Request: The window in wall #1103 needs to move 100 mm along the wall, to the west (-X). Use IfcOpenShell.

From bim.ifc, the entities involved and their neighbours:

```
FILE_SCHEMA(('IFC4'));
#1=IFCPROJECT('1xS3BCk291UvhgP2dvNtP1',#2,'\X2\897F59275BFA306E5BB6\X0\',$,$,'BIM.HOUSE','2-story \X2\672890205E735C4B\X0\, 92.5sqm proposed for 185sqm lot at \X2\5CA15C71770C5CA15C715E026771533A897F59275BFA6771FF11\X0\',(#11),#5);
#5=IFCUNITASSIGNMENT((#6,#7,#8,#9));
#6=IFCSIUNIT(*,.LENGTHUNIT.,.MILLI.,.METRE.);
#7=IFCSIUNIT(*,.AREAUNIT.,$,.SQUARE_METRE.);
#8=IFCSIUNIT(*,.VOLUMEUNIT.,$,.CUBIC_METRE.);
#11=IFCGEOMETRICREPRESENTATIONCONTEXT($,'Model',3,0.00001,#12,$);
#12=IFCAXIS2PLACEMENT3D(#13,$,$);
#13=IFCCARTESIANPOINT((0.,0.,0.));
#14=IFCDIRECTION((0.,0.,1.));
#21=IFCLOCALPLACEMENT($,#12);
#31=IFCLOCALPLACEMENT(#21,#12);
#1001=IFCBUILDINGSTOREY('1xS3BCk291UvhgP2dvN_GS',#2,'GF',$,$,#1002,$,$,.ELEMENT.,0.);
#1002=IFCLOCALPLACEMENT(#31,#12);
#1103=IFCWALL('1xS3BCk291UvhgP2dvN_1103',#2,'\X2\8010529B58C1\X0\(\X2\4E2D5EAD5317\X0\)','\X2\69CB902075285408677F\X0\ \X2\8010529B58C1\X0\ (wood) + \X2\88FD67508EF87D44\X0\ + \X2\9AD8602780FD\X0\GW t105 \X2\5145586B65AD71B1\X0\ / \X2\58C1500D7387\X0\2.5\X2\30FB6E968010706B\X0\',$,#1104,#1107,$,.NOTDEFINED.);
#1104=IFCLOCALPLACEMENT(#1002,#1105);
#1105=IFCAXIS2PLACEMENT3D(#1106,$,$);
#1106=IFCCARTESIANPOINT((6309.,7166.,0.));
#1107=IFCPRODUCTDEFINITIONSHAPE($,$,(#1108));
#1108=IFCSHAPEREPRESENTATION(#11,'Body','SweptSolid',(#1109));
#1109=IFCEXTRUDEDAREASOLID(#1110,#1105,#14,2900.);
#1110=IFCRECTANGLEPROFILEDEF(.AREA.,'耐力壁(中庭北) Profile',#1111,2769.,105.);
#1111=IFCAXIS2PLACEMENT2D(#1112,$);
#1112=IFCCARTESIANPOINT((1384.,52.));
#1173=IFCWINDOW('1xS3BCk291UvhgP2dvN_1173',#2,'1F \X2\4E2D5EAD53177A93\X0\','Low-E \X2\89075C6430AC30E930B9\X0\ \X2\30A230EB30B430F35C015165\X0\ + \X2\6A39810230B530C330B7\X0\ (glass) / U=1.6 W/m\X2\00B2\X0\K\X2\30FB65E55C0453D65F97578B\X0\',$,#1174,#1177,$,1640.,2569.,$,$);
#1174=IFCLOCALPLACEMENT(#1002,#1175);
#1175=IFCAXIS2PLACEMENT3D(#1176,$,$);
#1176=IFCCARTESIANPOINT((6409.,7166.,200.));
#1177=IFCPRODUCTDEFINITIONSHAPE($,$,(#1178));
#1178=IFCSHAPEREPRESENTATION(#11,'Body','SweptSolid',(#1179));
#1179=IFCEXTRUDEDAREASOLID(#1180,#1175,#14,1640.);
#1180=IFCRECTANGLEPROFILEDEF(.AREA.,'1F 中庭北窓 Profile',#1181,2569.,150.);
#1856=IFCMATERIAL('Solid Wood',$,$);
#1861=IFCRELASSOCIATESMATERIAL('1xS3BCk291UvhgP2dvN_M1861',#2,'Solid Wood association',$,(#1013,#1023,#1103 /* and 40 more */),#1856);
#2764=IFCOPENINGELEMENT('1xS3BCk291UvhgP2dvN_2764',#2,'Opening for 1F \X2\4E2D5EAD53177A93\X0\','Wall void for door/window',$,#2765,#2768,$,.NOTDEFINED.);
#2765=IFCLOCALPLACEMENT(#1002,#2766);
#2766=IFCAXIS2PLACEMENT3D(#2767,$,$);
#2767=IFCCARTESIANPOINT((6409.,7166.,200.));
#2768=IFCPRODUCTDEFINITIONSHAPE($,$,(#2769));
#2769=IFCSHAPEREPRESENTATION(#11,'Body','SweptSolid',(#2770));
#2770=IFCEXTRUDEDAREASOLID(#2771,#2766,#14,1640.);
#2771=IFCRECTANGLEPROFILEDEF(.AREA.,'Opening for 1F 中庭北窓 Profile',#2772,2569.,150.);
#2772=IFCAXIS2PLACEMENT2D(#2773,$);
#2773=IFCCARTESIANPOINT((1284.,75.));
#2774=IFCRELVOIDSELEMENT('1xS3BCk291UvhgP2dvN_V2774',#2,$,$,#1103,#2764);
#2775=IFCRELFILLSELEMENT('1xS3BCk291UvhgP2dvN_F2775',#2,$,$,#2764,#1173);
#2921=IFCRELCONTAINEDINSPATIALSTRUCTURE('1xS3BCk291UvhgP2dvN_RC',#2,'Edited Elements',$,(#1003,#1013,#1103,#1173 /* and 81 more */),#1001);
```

```python
import ifcopenshell
import ifcopenshell.api.geometry
import ifcopenshell.util.placement
import ifcopenshell.util.unit

model = ifcopenshell.open("bim.ifc")
unit_scale = ifcopenshell.util.unit.calculate_unit_scale(model)

window = model.by_guid("1xS3BCk291UvhgP2dvN_1173")
opening = window.FillsVoids[0].RelatingOpeningElement
wall = opening.VoidsElements[0].RelatingBuildingElement

wall_matrix = ifcopenshell.util.placement.get_local_placement(wall.ObjectPlacement)
shift = wall_matrix[:3, 0] * -0.1 / unit_scale
before = ifcopenshell.util.placement.get_local_placement(window.ObjectPlacement)[:3, 3].copy()

# The window is not placed relative to its opening, so move both.
for product in (opening, window):
    matrix = ifcopenshell.util.placement.get_local_placement(product.ObjectPlacement)
    matrix[:3, 3] += shift
    ifcopenshell.api.geometry.edit_object_placement(model, product=product, matrix=matrix, is_si=False)

after = ifcopenshell.util.placement.get_local_placement(window.ObjectPlacement)[:3, 3]
print("window moved by", (after - before).round(3) + 0.0)

model.write("bim-out.ifc")
```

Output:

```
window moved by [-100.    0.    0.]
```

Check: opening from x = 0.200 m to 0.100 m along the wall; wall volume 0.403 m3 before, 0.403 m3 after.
